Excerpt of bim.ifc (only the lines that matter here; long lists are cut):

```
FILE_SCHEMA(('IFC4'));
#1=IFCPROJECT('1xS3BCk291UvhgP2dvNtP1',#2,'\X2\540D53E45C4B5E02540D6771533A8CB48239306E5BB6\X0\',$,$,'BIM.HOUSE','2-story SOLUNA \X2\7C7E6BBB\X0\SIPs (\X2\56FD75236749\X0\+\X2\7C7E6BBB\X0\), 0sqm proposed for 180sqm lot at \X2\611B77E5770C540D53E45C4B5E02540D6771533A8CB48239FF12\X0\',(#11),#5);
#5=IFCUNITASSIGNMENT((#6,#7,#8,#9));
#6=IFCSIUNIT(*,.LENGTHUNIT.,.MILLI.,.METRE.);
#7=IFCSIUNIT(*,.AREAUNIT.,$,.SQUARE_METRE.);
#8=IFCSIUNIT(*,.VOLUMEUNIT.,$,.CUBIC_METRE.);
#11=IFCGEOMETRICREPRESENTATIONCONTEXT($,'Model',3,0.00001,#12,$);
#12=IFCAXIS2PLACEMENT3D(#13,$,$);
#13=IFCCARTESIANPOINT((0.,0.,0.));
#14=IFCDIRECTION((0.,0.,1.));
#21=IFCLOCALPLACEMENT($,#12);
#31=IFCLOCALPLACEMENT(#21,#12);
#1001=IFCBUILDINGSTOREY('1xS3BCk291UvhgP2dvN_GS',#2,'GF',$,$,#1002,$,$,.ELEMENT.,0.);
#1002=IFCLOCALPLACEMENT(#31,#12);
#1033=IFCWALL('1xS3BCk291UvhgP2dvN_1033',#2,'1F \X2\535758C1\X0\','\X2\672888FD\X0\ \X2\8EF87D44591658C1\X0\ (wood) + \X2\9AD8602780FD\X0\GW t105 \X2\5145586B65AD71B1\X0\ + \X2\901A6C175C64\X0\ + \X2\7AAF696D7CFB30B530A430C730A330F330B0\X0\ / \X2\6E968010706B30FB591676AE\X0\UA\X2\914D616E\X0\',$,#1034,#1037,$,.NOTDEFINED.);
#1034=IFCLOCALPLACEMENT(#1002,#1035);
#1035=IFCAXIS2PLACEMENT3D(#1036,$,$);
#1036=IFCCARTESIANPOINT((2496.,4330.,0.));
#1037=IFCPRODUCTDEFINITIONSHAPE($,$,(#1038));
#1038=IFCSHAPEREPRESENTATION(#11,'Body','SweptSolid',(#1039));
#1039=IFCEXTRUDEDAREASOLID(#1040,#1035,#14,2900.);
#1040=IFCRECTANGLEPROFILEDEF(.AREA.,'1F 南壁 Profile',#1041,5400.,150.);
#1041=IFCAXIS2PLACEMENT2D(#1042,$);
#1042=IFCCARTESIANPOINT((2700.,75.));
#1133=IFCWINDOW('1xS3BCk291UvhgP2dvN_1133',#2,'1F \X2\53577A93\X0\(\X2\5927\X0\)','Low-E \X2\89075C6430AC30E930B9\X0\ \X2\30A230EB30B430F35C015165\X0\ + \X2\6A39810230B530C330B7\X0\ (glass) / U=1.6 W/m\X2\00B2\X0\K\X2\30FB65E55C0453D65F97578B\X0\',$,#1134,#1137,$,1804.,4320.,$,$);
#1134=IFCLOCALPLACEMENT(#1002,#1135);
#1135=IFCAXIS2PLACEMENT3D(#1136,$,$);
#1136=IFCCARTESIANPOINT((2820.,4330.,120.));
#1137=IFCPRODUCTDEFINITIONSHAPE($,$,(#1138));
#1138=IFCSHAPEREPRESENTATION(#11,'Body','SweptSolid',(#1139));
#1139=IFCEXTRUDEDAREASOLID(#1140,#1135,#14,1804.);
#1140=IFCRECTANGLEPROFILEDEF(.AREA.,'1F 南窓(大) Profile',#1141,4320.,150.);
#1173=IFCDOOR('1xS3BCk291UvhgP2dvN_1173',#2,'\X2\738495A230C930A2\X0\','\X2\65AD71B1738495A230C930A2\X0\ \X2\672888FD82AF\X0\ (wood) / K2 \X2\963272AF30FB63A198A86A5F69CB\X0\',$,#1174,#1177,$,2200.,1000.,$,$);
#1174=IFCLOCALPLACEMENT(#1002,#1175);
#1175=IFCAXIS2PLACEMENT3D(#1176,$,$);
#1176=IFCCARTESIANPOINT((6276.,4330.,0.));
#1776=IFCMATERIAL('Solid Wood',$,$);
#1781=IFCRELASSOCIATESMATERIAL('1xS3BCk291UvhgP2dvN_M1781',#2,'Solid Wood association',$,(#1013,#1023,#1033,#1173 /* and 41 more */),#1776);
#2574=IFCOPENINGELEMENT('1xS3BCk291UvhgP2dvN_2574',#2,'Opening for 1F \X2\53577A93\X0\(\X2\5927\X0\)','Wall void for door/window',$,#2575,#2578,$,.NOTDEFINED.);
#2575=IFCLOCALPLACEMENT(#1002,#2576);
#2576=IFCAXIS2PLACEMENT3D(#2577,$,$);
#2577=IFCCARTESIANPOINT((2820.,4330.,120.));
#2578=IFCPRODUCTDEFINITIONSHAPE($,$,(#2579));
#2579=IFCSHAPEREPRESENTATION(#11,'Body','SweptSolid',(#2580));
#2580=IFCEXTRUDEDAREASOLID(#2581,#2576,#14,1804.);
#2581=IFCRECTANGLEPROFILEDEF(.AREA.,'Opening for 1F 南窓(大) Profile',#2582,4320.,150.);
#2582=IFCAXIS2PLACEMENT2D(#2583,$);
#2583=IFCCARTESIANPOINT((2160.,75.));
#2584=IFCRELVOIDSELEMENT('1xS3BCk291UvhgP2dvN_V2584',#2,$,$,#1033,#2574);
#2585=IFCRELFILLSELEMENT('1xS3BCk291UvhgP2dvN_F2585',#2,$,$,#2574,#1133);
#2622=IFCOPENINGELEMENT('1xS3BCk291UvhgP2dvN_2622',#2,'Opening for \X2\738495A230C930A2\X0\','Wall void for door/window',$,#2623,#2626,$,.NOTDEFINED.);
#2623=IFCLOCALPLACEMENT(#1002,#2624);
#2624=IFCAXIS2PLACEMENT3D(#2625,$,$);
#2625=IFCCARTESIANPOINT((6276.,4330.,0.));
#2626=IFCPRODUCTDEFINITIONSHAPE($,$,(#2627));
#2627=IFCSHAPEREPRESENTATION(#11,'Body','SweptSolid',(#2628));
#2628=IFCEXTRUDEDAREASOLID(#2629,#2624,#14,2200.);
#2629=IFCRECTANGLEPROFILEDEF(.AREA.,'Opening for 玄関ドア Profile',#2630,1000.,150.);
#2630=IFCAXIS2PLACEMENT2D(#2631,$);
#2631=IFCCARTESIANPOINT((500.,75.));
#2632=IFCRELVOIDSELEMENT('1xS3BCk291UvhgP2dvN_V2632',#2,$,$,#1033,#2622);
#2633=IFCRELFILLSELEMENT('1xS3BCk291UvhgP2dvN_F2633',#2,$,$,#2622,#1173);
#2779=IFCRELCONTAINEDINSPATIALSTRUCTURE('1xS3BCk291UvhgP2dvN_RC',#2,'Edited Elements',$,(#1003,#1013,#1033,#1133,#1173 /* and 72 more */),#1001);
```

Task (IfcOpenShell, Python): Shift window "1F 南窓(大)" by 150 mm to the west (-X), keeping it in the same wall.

```python
import ifcopenshell
import ifcopenshell.api.geometry
import ifcopenshell.util.placement
import ifcopenshell.util.unit

model = ifcopenshell.open("bim.ifc")
unit_scale = ifcopenshell.util.unit.calculate_unit_scale(model)

window = model.by_guid("1xS3BCk291UvhgP2dvN_1133")
opening = window.FillsVoids[0].RelatingOpeningElement
wall = opening.VoidsElements[0].RelatingBuildingElement

wall_matrix = ifcopenshell.util.placement.get_local_placement(wall.ObjectPlacement)
shift = wall_matrix[:3, 0] * -0.15 / unit_scale
before = ifcopenshell.util.placement.get_local_placement(window.ObjectPlacement)[:3, 3].copy()

# The window is not placed relative to its opening, so move both.
for product in (opening, window):
    matrix = ifcopenshell.util.placement.get_local_placement(product.ObjectPlacement)
    matrix[:3, 3] += shift
    ifcopenshell.api.geometry.edit_object_placement(model, product=product, matrix=matrix, is_si=False)

after = ifcopenshell.util.placement.get_local_placement(window.ObjectPlacement)[:3, 3]
print("window moved by", (after - before).round(3) + 0.0)

model.write("bim_updated.ifc")
```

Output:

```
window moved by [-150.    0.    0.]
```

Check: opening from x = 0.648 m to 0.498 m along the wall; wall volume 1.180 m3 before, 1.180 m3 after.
